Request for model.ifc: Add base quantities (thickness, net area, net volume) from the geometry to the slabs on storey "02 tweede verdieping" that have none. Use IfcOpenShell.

First a look at what the model holds.

```python
import ifcopenshell
import ifcopenshell.util.element
import ifcopenshell.util.unit

model = ifcopenshell.open("model.ifc")
print(model.schema)
for unit_type in ("LENGTHUNIT", "AREAUNIT", "VOLUMEUNIT"):
    print(unit_type, ifcopenshell.util.unit.calculate_unit_scale(model, unit_type))
storey = next(s for s in model.by_type("IfcBuildingStorey") if s.Name == "02 tweede verdieping")
slabs = [e for e in ifcopenshell.util.element.get_decomposition(storey) if e.is_a("IfcSlab")]
for e in sorted(slabs, key=lambda e: e.id()):
    print(e.id(), e.is_a(), e.Name, list(ifcopenshell.util.element.get_psets(e, qtos_only=True)), sep=" | ")
```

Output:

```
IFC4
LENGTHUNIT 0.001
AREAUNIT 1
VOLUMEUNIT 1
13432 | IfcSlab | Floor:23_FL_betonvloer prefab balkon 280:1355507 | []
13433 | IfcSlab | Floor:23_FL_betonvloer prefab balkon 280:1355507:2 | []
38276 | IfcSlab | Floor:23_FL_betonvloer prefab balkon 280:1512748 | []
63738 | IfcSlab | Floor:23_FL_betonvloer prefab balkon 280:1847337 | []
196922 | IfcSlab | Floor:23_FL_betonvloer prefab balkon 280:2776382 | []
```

```python
import ifcopenshell
import ifcopenshell.api.pset
import ifcopenshell.geom
import ifcopenshell.util.element
import ifcopenshell.util.shape
import ifcopenshell.util.unit

model = ifcopenshell.open("model.ifc")
unit_scale = ifcopenshell.util.unit.calculate_unit_scale(model)
area_scale = ifcopenshell.util.unit.calculate_unit_scale(model, "AREAUNIT")
volume_scale = ifcopenshell.util.unit.calculate_unit_scale(model, "VOLUMEUNIT")
settings = ifcopenshell.geom.settings()

storey = next(s for s in model.by_type("IfcBuildingStorey") if s.Name == "02 tweede verdieping")
slabs = [e for e in ifcopenshell.util.element.get_decomposition(storey) if e.is_a("IfcSlab")]

for e in sorted(slabs, key=lambda e: e.id()):
    if ifcopenshell.util.element.get_psets(e, qtos_only=True, should_inherit=False):
        continue
    # Geometry comes back in metres, in the element's own axes.
    shape = ifcopenshell.geom.create_shape(settings, e)
    values = {
        "Width": ifcopenshell.util.shape.get_z(shape.geometry) / unit_scale,
        "NetArea": ifcopenshell.util.shape.get_footprint_area(shape.geometry) / area_scale,
        "NetVolume": ifcopenshell.util.shape.get_volume(shape.geometry) / volume_scale,
    }
    qto = ifcopenshell.api.pset.add_qto(model, product=e, name="Qto_SlabBaseQuantities")
    ifcopenshell.api.pset.edit_qto(model, qto=qto, properties=values)
    print(e.id(), {k: round(v, 3) for k, v in values.items()})

model.write("model_rev.ifc")
```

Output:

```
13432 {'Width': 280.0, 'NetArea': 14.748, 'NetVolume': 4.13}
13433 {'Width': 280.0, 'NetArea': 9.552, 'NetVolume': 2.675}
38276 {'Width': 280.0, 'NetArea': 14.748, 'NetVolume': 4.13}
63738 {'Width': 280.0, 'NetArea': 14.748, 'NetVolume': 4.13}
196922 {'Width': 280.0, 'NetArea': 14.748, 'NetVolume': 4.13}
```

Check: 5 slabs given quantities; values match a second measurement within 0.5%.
